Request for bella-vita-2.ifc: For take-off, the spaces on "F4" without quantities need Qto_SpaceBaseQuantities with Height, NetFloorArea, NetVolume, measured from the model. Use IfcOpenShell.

First a look at what the model holds.

```python
import ifcopenshell
import ifcopenshell.util.element
import ifcopenshell.util.unit

model = ifcopenshell.open("bella-vita-2.ifc")
print(model.schema)
for unit_type in ("LENGTHUNIT", "AREAUNIT", "VOLUMEUNIT"):
    print(unit_type, ifcopenshell.util.unit.calculate_unit_scale(model, unit_type))
storey = next(s for s in model.by_type("IfcBuildingStorey") if s.Name == "F4")
spaces = [e for e in ifcopenshell.util.element.get_decomposition(storey) if e.is_a("IfcSpace")]
for e in sorted(spaces, key=lambda e: e.id()):
    print(e.id(), e.is_a(), e.Name, list(ifcopenshell.util.element.get_psets(e, qtos_only=True)), sep=" | ")
```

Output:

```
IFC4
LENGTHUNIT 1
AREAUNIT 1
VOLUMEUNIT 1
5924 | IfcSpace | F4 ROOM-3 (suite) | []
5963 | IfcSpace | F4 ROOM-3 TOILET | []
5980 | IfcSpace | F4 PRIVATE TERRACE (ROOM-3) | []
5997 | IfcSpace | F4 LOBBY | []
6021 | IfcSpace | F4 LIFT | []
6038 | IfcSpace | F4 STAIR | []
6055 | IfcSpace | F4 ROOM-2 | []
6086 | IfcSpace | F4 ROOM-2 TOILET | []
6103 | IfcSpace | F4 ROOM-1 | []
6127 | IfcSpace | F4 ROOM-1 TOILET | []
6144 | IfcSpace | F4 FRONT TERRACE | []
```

```python
import ifcopenshell
import ifcopenshell.api.pset
import ifcopenshell.geom
import ifcopenshell.util.element
import ifcopenshell.util.shape
import ifcopenshell.util.unit

model = ifcopenshell.open("bella-vita-2.ifc")
unit_scale = ifcopenshell.util.unit.calculate_unit_scale(model)
area_scale = ifcopenshell.util.unit.calculate_unit_scale(model, "AREAUNIT")
volume_scale = ifcopenshell.util.unit.calculate_unit_scale(model, "VOLUMEUNIT")
settings = ifcopenshell.geom.settings()

storey = next(s for s in model.by_type("IfcBuildingStorey") if s.Name == "F4")
spaces = [e for e in ifcopenshell.util.element.get_decomposition(storey) if e.is_a("IfcSpace")]

for e in sorted(spaces, key=lambda e: e.id()):
    if ifcopenshell.util.element.get_psets(e, qtos_only=True, should_inherit=False):
        continue
    # Geometry comes back in metres, in the element's own axes.
    shape = ifcopenshell.geom.create_shape(settings, e)
    values = {
        "Height": ifcopenshell.util.shape.get_z(shape.geometry) / unit_scale,
        "NetFloorArea": ifcopenshell.util.shape.get_footprint_area(shape.geometry) / area_scale,
        "NetVolume": ifcopenshell.util.shape.get_volume(shape.geometry) / volume_scale,
    }
    qto = ifcopenshell.api.pset.add_qto(model, product=e, name="Qto_SpaceBaseQuantities")
    ifcopenshell.api.pset.edit_qto(model, qto=qto, properties=values)
    print(e.id(), {k: round(v, 3) for k, v in values.items()})

model.write("bella-vita-2-out.ifc")
```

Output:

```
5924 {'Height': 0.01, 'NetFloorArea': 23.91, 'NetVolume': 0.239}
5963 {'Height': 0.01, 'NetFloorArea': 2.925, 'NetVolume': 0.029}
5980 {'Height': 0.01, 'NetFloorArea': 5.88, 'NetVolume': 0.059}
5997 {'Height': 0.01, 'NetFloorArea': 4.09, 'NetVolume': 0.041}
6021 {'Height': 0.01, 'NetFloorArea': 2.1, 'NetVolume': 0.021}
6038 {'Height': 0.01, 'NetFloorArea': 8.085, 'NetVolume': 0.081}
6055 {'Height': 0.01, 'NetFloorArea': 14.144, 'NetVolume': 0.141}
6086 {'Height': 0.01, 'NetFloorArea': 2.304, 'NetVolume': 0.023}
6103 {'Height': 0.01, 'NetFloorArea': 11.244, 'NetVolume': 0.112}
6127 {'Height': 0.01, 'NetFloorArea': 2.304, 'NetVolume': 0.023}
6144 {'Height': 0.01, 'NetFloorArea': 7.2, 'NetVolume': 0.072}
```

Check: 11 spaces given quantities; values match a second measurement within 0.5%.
